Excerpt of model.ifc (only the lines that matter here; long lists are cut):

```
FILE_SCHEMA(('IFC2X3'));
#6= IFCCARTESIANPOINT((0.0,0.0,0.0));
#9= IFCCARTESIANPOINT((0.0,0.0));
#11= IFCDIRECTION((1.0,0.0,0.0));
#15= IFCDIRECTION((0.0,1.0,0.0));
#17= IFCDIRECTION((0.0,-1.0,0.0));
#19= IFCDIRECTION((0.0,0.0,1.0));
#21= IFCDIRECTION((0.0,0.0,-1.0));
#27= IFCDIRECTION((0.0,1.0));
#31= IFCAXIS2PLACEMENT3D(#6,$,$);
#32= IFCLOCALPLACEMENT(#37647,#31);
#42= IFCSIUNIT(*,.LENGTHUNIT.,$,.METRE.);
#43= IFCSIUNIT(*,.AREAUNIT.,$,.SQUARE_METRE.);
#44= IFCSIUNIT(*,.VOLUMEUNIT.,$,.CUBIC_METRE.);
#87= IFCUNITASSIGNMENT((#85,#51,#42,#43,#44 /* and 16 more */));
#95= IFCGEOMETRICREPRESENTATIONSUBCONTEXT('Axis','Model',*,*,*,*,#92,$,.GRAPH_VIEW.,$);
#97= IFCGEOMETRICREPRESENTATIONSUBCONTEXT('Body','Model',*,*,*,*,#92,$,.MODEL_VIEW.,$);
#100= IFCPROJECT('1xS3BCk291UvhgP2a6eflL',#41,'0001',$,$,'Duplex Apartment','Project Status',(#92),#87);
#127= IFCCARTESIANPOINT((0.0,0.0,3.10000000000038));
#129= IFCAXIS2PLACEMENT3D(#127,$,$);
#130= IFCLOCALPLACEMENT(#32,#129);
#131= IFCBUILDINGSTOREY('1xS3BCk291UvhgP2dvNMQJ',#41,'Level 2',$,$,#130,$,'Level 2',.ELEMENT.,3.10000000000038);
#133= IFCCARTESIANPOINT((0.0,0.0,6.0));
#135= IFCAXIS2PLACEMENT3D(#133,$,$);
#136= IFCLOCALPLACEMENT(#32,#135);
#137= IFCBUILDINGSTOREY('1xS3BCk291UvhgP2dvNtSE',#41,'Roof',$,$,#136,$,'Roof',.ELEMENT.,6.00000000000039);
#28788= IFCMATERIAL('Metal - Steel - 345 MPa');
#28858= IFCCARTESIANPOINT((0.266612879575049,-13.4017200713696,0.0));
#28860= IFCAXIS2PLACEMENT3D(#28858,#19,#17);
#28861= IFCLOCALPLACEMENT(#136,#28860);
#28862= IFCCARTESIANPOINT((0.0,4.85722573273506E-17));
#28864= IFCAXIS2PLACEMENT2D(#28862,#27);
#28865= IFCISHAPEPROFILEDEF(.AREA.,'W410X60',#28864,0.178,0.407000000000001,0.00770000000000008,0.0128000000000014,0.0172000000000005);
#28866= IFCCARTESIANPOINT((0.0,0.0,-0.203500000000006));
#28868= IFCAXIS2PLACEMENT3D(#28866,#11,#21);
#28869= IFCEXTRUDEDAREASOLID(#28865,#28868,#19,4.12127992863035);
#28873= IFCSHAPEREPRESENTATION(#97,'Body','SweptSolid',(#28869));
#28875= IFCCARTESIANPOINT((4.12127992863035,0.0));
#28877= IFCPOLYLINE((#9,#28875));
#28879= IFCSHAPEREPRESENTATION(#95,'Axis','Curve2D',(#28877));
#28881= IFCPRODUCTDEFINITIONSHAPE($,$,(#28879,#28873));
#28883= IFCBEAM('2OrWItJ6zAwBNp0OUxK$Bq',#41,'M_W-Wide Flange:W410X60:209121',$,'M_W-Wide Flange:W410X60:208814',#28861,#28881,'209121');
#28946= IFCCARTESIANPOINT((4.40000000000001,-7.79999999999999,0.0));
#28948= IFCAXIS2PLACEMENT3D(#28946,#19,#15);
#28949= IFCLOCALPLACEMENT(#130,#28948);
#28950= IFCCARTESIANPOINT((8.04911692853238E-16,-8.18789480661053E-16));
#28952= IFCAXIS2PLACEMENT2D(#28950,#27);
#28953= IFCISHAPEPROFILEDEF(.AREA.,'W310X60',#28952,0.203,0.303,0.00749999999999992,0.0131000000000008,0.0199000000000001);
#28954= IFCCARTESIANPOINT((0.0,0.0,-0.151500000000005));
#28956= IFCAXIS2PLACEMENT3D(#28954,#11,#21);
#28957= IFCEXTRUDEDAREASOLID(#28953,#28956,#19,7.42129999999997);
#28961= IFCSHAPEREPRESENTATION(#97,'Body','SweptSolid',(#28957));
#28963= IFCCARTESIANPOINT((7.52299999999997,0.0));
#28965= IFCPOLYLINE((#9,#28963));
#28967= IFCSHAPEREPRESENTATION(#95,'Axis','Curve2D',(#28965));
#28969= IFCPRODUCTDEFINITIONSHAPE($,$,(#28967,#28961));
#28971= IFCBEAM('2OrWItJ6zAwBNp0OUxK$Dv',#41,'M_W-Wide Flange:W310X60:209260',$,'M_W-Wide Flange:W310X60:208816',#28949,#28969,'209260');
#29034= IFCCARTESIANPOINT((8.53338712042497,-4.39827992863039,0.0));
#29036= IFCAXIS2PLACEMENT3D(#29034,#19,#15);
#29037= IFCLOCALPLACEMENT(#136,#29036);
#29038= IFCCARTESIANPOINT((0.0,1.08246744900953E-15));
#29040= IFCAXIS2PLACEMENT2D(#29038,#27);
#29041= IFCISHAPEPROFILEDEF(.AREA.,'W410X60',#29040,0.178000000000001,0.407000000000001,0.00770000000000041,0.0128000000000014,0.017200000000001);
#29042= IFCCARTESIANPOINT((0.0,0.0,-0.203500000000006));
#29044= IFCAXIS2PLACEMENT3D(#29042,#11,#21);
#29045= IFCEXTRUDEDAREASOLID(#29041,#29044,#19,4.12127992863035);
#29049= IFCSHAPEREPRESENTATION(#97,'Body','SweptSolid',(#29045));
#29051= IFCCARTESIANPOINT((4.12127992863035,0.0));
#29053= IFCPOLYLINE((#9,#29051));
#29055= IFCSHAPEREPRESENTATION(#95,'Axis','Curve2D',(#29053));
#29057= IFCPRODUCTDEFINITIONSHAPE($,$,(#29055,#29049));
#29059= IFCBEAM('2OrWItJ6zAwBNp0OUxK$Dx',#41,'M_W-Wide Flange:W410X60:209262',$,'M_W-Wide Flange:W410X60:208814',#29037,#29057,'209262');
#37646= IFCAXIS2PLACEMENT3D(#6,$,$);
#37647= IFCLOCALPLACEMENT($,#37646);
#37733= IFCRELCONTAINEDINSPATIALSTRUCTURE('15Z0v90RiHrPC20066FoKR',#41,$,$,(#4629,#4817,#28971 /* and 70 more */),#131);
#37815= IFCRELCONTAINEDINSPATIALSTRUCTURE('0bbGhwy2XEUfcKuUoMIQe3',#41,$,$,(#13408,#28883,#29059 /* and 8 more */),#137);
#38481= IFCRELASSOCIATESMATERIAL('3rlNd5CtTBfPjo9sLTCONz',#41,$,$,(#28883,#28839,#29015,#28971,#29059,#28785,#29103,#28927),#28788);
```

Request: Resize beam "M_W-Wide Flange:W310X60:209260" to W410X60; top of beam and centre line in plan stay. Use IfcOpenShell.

```python
import ifcopenshell
import ifcopenshell.util.element
import ifcopenshell.util.representation

model = ifcopenshell.open("model.ifc")

member = model.by_guid("2OrWItJ6zAwBNp0OUxK$Dv")
source = next(p for p in model.by_type("IfcIShapeProfileDef") if p.ProfileName == "W410X60")

body = ifcopenshell.util.representation.get_representation(member, "Model", "Body")
solid = body.Items[0]
old_profile = solid.SweptArea

# Copy the section's sizes but keep this member's own profile position.
profile = ifcopenshell.util.element.copy(model, source)
# Profiles are centred, so shift by half the change in depth to hold the top.
shift = (old_profile.OverallDepth - profile.OverallDepth) / 2
x, y = old_profile.Position.Location.Coordinates
up = (-1.0, 0.0)  # upwards, in the solid's own plane
location = model.createIfcCartesianPoint((x + up[0] * shift, y + up[1] * shift))
profile.Position = model.createIfcAxis2Placement2D(location, old_profile.Position.RefDirection)
solid.SweptArea = profile
if not model.get_total_inverses(old_profile):
    ifcopenshell.util.element.remove_deep2(model, old_profile)
member.Name = member.Name.replace("W310X60", "W410X60")
member.ObjectType = member.ObjectType.replace("W310X60", "W410X60")

print(solid.SweptArea)

model.write("model_rev.ifc")
```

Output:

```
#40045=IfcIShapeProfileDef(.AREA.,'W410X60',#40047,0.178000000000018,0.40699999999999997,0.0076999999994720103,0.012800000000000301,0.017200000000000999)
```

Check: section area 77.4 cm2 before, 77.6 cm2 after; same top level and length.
